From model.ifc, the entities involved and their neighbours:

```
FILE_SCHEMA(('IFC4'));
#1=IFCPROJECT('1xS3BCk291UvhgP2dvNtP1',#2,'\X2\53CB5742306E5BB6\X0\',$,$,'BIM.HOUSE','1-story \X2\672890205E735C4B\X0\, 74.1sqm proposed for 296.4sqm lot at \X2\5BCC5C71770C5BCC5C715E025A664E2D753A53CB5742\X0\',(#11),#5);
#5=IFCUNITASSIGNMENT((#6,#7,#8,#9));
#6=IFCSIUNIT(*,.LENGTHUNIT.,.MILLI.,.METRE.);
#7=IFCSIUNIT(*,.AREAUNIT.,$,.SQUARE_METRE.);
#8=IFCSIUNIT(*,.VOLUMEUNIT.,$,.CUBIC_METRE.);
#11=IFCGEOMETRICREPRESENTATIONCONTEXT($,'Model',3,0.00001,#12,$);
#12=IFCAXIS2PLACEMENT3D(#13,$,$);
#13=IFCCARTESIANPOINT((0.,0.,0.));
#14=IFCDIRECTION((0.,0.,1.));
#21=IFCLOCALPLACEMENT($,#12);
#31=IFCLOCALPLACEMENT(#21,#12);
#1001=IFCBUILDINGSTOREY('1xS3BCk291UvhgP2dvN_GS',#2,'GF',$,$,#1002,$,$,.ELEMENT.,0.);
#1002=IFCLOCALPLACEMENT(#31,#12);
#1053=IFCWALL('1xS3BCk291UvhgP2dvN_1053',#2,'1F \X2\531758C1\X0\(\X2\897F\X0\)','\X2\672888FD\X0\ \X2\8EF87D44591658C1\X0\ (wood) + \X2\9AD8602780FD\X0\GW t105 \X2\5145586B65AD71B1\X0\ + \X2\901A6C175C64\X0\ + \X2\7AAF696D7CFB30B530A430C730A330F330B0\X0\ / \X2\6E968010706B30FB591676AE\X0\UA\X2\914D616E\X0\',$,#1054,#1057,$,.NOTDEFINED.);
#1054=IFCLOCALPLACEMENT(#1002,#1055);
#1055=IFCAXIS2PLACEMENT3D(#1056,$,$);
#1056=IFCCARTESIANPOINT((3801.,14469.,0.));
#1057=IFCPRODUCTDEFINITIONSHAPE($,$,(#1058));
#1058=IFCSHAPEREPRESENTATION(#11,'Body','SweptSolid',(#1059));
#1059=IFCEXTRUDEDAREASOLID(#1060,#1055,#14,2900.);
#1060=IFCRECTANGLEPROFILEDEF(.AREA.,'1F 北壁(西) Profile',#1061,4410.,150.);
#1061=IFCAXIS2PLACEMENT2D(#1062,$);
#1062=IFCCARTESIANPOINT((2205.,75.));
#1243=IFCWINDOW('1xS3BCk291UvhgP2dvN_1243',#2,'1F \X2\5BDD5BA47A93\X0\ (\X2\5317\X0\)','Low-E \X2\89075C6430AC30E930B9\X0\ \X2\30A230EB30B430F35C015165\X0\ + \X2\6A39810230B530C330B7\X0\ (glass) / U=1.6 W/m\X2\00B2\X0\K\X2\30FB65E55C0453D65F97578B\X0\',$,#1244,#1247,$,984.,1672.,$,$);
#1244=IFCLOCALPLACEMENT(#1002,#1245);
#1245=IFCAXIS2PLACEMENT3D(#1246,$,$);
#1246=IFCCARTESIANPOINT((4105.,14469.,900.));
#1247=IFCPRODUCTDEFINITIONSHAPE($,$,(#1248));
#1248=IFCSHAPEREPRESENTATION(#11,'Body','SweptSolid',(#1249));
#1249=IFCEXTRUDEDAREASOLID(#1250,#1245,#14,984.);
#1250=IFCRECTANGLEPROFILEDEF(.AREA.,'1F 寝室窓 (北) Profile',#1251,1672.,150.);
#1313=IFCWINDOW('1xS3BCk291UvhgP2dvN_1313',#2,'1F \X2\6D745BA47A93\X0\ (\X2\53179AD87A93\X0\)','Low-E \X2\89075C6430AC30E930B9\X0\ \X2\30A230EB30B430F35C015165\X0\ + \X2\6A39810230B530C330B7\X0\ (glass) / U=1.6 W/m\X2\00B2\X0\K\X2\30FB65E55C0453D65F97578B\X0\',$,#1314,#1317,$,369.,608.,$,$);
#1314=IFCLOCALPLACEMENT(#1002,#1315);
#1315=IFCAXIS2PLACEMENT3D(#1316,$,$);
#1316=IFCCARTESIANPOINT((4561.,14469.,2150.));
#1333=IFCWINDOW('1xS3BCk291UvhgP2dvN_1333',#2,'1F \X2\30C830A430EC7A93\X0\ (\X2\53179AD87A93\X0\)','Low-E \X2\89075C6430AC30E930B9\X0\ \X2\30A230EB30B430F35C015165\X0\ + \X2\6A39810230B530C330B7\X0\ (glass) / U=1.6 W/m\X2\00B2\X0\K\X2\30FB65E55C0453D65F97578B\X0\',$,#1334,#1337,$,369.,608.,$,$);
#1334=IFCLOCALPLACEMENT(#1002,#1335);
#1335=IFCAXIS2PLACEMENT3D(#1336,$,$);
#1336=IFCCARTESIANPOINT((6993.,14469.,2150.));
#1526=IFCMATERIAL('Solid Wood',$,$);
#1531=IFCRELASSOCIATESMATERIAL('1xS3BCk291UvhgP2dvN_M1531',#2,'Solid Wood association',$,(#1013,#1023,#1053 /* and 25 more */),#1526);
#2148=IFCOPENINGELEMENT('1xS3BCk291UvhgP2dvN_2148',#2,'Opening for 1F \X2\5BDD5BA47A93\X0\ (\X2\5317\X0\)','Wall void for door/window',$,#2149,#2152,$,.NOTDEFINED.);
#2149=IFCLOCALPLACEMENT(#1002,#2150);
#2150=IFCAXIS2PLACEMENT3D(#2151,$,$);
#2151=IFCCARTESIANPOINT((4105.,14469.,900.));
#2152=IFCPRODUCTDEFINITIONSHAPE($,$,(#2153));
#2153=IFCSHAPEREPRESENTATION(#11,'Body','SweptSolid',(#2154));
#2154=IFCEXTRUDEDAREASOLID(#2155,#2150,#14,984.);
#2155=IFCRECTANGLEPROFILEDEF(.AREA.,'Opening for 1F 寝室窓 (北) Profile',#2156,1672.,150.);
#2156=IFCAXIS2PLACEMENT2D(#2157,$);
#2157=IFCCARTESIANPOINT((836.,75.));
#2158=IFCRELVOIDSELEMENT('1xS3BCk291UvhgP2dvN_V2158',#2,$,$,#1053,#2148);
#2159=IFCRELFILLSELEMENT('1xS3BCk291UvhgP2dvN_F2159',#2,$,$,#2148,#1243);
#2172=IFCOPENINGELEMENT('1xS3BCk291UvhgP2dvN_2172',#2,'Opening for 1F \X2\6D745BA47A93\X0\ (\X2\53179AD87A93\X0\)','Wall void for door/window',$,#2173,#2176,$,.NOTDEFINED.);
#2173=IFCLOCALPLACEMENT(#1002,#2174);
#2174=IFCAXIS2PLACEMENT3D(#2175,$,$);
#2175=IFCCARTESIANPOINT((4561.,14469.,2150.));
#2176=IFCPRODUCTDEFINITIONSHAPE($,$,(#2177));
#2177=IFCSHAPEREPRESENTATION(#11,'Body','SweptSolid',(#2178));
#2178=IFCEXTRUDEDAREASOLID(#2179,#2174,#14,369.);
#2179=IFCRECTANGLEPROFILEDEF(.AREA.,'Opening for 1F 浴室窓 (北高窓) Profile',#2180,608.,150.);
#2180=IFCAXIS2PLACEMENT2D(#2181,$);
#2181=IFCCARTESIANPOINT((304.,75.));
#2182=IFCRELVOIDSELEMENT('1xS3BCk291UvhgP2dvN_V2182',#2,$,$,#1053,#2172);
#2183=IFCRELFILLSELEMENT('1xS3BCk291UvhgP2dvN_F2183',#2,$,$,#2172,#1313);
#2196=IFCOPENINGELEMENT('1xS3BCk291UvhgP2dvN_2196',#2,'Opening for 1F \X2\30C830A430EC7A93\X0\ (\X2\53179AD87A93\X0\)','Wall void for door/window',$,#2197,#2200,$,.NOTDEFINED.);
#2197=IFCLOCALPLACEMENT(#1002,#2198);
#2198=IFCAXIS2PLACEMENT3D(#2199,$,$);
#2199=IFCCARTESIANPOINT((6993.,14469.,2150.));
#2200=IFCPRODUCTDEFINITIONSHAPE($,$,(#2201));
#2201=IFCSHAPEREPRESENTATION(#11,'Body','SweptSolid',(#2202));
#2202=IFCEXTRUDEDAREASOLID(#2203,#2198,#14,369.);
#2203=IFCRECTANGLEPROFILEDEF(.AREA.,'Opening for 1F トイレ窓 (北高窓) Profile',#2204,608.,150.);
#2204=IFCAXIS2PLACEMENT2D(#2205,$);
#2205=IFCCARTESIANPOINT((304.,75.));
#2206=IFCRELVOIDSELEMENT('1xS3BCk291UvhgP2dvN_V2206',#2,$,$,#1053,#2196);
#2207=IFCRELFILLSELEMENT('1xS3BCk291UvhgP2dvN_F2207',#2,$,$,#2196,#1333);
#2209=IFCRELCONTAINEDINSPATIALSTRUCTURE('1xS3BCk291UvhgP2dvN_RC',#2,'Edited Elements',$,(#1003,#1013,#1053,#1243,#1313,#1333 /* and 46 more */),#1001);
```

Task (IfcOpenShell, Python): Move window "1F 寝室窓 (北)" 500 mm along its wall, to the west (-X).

```python
import ifcopenshell
import ifcopenshell.api.geometry
import ifcopenshell.util.placement
import ifcopenshell.util.unit

model = ifcopenshell.open("model.ifc")
unit_scale = ifcopenshell.util.unit.calculate_unit_scale(model)

window = model.by_guid("1xS3BCk291UvhgP2dvN_1243")
opening = window.FillsVoids[0].RelatingOpeningElement
wall = opening.VoidsElements[0].RelatingBuildingElement

wall_matrix = ifcopenshell.util.placement.get_local_placement(wall.ObjectPlacement)
shift = wall_matrix[:3, 0] * -0.5 / unit_scale
before = ifcopenshell.util.placement.get_local_placement(window.ObjectPlacement)[:3, 3].copy()

# The window is not placed relative to its opening, so move both.
for product in (opening, window):
    matrix = ifcopenshell.util.placement.get_local_placement(product.ObjectPlacement)
    matrix[:3, 3] += shift
    ifcopenshell.api.geometry.edit_object_placement(model, product=product, matrix=matrix, is_si=False)

after = ifcopenshell.util.placement.get_local_placement(window.ObjectPlacement)[:3, 3]
print("window moved by", (after - before).round(3) + 0.0)

model.write("model_updated.ifc")
```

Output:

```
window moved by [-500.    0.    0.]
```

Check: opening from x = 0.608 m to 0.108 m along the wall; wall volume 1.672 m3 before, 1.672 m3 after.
